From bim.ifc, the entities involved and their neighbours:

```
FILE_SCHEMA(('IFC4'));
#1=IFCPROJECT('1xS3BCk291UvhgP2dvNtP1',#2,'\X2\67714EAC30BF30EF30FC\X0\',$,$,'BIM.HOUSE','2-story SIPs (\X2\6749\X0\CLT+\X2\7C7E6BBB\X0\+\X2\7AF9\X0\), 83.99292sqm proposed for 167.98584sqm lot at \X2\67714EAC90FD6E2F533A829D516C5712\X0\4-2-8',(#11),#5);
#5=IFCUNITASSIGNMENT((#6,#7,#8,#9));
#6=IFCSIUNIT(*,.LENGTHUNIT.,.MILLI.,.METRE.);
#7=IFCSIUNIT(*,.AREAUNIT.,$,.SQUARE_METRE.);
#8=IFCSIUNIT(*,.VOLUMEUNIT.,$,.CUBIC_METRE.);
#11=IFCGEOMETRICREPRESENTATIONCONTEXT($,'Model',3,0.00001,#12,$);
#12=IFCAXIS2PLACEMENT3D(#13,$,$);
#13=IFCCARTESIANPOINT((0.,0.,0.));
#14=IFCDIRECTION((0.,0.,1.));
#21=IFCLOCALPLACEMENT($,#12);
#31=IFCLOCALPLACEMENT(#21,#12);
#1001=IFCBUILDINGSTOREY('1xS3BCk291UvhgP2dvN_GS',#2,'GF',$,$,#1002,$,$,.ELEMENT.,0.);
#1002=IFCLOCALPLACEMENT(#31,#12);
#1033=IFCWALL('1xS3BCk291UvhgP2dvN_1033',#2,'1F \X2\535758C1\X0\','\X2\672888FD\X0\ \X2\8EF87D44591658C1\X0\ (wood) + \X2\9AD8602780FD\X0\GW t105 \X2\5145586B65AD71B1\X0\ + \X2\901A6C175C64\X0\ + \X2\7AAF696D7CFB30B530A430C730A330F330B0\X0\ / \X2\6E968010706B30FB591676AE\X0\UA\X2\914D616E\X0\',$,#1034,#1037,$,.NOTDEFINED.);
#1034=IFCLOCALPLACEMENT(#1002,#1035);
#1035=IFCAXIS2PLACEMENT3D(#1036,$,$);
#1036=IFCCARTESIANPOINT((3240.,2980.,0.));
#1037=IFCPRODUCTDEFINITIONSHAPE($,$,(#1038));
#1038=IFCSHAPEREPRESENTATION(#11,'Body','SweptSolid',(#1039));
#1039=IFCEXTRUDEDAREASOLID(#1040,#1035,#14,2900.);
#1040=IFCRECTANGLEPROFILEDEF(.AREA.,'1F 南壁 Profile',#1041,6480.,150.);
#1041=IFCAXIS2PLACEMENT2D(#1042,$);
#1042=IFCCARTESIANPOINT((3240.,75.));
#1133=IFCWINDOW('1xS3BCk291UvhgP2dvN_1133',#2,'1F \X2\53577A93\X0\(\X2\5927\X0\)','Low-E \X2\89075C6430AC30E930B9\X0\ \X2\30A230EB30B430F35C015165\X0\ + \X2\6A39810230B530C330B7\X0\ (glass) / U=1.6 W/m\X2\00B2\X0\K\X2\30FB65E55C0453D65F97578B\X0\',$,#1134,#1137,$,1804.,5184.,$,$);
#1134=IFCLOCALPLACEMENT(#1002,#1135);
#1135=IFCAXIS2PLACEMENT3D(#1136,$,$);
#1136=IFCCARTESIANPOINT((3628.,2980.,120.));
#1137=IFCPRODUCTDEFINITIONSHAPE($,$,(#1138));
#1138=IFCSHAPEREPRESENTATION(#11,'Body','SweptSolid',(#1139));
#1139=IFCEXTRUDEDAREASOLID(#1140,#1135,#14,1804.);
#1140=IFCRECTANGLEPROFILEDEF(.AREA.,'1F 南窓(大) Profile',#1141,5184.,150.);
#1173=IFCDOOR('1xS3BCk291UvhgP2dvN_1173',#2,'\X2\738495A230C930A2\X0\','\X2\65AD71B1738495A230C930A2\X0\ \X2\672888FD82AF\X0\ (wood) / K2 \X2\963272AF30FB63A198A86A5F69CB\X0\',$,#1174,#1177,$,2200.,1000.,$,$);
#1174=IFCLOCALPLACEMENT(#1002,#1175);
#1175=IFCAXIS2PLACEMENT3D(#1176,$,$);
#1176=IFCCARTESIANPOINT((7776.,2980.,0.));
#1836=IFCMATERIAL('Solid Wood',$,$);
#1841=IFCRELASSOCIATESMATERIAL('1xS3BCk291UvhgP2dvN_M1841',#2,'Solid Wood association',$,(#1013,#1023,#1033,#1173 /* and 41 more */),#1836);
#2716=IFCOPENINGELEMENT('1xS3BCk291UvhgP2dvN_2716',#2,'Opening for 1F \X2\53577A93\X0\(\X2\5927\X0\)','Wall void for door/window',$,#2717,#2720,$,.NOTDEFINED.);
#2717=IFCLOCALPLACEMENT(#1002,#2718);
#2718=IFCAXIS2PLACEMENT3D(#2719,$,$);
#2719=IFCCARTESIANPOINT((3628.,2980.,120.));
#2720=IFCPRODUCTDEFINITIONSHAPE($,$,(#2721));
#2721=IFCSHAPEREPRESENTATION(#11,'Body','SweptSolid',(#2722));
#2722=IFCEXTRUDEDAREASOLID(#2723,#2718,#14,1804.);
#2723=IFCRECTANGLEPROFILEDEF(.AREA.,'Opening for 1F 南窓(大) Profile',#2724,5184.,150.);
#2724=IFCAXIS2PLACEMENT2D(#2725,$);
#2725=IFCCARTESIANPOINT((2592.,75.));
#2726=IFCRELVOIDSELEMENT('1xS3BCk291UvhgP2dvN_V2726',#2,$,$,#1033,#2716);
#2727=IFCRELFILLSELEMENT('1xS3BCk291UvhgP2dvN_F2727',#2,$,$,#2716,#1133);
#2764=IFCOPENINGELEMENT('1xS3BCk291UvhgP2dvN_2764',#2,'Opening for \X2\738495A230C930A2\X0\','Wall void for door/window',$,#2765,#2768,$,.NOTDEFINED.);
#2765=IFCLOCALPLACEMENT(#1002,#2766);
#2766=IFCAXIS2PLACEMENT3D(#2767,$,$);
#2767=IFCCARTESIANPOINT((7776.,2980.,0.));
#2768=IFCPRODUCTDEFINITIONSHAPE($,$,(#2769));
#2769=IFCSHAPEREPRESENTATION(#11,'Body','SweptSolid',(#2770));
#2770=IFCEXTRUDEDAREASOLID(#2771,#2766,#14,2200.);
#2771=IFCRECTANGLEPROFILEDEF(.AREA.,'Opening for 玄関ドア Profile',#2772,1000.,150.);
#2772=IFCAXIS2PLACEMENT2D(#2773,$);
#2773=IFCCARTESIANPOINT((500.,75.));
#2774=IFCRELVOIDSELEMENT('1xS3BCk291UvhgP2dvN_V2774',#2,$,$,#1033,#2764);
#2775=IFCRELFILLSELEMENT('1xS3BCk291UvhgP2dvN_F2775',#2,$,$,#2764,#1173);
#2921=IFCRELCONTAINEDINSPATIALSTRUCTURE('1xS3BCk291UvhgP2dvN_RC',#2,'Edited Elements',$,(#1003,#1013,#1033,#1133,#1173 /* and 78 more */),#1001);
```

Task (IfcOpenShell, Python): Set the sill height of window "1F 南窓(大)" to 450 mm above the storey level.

```python
import numpy as np
import ifcopenshell
import ifcopenshell.api.geometry
import ifcopenshell.geom
import ifcopenshell.util.element
import ifcopenshell.util.placement
import ifcopenshell.util.shape
import ifcopenshell.util.unit

model = ifcopenshell.open("bim.ifc")
unit_scale = ifcopenshell.util.unit.calculate_unit_scale(model)

window = model.by_guid("1xS3BCk291UvhgP2dvN_1133")
opening = window.FillsVoids[0].RelatingOpeningElement
storey = ifcopenshell.util.element.get_container(window, ifc_class="IfcBuildingStorey")
level = ifcopenshell.util.placement.get_local_placement(storey.ObjectPlacement)[2, 3]

# The opening's origin need not be at the sill, so measure its lowest point.
shape = ifcopenshell.geom.create_shape(ifcopenshell.geom.settings(), opening)
bottom = ifcopenshell.util.shape.get_shape_bottom_elevation(shape, shape.geometry) / unit_scale
dz = level + 450.0 - bottom

shift = np.array([0.0, 0.0, dz])
# The window is not placed relative to its opening, so move both.
for product in (opening, window):
    matrix = ifcopenshell.util.placement.get_local_placement(product.ObjectPlacement)
    matrix[:3, 3] += shift
    ifcopenshell.api.geometry.edit_object_placement(model, product=product, matrix=matrix, is_si=False)

print(f"moved by {dz * unit_scale:+.3f} m")

model.write("bim-out.ifc")
```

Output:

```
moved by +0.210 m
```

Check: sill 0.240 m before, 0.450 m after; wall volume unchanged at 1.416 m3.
